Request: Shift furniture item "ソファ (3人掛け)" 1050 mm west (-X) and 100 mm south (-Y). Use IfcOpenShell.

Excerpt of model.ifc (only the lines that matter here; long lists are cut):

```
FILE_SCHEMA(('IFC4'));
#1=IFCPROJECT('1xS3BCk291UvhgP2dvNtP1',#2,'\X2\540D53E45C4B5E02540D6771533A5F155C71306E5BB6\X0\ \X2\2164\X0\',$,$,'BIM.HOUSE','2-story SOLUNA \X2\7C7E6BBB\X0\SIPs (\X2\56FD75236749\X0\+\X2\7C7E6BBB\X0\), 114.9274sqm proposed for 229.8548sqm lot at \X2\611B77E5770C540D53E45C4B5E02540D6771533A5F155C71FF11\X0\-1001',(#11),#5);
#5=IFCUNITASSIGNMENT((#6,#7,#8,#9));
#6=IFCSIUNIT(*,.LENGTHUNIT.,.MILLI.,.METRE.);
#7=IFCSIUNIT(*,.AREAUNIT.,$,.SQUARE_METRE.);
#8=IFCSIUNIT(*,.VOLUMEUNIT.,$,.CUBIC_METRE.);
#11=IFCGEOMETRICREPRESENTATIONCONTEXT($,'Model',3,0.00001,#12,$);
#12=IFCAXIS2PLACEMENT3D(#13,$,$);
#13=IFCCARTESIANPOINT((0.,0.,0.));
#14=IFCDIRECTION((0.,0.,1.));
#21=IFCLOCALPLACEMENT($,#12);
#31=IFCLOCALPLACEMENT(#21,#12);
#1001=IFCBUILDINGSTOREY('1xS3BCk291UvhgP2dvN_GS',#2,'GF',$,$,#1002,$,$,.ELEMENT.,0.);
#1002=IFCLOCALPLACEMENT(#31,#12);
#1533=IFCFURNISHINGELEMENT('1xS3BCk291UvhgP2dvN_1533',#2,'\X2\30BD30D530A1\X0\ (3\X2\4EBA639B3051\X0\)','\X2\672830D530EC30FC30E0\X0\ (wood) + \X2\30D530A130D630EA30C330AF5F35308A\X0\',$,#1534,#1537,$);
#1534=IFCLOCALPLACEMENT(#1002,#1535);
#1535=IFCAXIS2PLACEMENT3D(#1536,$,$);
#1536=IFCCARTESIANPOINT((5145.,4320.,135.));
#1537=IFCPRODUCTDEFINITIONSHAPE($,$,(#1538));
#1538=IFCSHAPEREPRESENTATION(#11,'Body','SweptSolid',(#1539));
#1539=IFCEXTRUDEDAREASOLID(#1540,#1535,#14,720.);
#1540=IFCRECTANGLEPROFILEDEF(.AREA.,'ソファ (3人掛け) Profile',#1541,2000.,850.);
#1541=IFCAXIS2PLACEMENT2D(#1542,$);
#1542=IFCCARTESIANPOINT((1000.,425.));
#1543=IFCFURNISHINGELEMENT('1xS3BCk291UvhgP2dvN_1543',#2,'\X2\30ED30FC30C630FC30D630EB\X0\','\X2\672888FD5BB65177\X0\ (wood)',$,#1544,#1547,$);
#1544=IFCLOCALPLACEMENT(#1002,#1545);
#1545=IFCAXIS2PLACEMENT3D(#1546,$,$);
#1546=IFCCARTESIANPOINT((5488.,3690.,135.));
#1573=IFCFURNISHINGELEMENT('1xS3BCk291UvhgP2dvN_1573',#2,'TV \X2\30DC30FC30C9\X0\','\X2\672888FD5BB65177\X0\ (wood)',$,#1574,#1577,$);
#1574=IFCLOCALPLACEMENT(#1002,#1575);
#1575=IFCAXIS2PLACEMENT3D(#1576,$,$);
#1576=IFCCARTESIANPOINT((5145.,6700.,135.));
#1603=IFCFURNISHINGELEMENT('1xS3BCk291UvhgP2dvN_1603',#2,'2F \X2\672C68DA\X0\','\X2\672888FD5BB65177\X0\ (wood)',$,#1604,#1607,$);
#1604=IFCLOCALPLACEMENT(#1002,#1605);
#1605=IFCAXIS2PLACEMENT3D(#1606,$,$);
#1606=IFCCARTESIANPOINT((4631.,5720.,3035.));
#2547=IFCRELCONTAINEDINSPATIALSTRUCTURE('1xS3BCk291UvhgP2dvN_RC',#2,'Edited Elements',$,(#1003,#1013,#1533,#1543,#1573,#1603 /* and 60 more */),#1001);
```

```python
import ifcopenshell
import ifcopenshell.api.geometry
import ifcopenshell.util.placement

model = ifcopenshell.open("model.ifc")

item = model.by_guid("1xS3BCk291UvhgP2dvN_1533")
matrix = ifcopenshell.util.placement.get_local_placement(item.ObjectPlacement)
matrix[0, 3] -= 1050.0
matrix[1, 3] -= 100.0
ifcopenshell.api.geometry.edit_object_placement(model, product=item, matrix=matrix, is_si=False)

print(ifcopenshell.util.placement.get_local_placement(item.ObjectPlacement).round(3) + 0.0)

model.write("model-out.ifc")
```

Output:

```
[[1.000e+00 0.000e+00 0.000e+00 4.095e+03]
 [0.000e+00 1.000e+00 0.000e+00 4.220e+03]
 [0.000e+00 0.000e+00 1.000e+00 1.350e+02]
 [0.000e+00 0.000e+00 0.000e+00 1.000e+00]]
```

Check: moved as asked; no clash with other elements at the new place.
